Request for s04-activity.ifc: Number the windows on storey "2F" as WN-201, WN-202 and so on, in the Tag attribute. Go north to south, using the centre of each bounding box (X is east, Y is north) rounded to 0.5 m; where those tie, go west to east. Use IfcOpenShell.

First a look at what the model holds.

```python
import ifcopenshell
import ifcopenshell.util.element
import ifcopenshell.util.placement

model = ifcopenshell.open("s04-activity.ifc")
print(model.schema)
storey = next(s for s in model.by_type("IfcBuildingStorey") if s.Name == "2F")
windows = [e for e in ifcopenshell.util.element.get_decomposition(storey) if e.is_a("IfcWindow")]
for e in sorted(windows, key=lambda e: e.id()):
    origin = ifcopenshell.util.placement.get_local_placement(e.ObjectPlacement)[:3, 3]
    print(e.id(), e.Tag, e.Name, origin.round(2) + 0.0, sep=" | ")
```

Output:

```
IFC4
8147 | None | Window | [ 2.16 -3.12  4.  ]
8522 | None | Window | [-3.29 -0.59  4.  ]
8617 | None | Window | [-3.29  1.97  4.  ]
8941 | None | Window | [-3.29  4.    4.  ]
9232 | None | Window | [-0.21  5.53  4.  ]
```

```python
import ifcopenshell
import ifcopenshell.geom
import ifcopenshell.util.element
import ifcopenshell.util.shape

model = ifcopenshell.open("s04-activity.ifc")
settings = ifcopenshell.geom.settings()
settings.set("use-world-coords", True)


def centre(element):
    shape = ifcopenshell.geom.create_shape(settings, element)
    return ifcopenshell.util.shape.get_bbox_centroid(shape.geometry)


storey = next(s for s in model.by_type("IfcBuildingStorey") if s.Name == "2F")
windows = [e for e in ifcopenshell.util.element.get_decomposition(storey) if e.is_a("IfcWindow")]

# Insertion points can sit at a corner or the storey origin, so sort by the geometry (in metres).
centres = {e: centre(e) for e in windows}
windows.sort(key=lambda e: (-round(centres[e][1] / 0.5), centres[e][0]))

for i, e in enumerate(windows, start=1):
    number = f"WN-2{i:02d}"
    e.Tag = number
    print(e.id(), number)

model.write("s04-activity_updated.ifc")
```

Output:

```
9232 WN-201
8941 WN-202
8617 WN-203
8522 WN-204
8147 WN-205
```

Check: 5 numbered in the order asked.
